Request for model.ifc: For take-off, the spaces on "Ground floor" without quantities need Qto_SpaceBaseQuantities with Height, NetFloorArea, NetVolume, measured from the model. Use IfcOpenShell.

First a look at what the model holds.

```python
import ifcopenshell
import ifcopenshell.util.element
import ifcopenshell.util.unit

model = ifcopenshell.open("model.ifc")
print(model.schema)
for unit_type in ("LENGTHUNIT", "AREAUNIT", "VOLUMEUNIT"):
    print(unit_type, ifcopenshell.util.unit.calculate_unit_scale(model, unit_type))
storey = next(s for s in model.by_type("IfcBuildingStorey") if s.Name == "Ground floor")
spaces = [e for e in ifcopenshell.util.element.get_decomposition(storey) if e.is_a("IfcSpace")]
for e in sorted(spaces, key=lambda e: e.id()):
    print(e.id(), e.is_a(), e.Name, list(ifcopenshell.util.element.get_psets(e, qtos_only=True)), sep=" | ")
```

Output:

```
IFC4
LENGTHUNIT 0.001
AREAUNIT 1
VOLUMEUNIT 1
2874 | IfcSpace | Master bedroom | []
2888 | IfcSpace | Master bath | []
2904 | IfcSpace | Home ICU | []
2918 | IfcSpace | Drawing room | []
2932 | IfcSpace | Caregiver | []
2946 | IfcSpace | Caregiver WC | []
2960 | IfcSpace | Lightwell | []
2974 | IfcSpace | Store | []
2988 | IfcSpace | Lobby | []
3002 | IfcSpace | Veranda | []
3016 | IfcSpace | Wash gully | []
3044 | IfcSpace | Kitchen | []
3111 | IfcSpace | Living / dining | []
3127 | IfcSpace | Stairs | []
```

```python
import ifcopenshell
import ifcopenshell.api.pset
import ifcopenshell.geom
import ifcopenshell.util.element
import ifcopenshell.util.shape
import ifcopenshell.util.unit

model = ifcopenshell.open("model.ifc")
unit_scale = ifcopenshell.util.unit.calculate_unit_scale(model)
area_scale = ifcopenshell.util.unit.calculate_unit_scale(model, "AREAUNIT")
volume_scale = ifcopenshell.util.unit.calculate_unit_scale(model, "VOLUMEUNIT")
settings = ifcopenshell.geom.settings()

storey = next(s for s in model.by_type("IfcBuildingStorey") if s.Name == "Ground floor")
spaces = [e for e in ifcopenshell.util.element.get_decomposition(storey) if e.is_a("IfcSpace")]

for e in sorted(spaces, key=lambda e: e.id()):
    if ifcopenshell.util.element.get_psets(e, qtos_only=True, should_inherit=False):
        continue
    # Geometry comes back in metres, in the element's own axes.
    shape = ifcopenshell.geom.create_shape(settings, e)
    values = {
        "Height": ifcopenshell.util.shape.get_z(shape.geometry) / unit_scale,
        "NetFloorArea": ifcopenshell.util.shape.get_footprint_area(shape.geometry) / area_scale,
        "NetVolume": ifcopenshell.util.shape.get_volume(shape.geometry) / volume_scale,
    }
    qto = ifcopenshell.api.pset.add_qto(model, product=e, name="Qto_SpaceBaseQuantities")
    ifcopenshell.api.pset.edit_qto(model, qto=qto, properties=values)
    print(e.id(), {k: round(v, 3) for k, v in values.items()})

model.write("model_updated.ifc")
```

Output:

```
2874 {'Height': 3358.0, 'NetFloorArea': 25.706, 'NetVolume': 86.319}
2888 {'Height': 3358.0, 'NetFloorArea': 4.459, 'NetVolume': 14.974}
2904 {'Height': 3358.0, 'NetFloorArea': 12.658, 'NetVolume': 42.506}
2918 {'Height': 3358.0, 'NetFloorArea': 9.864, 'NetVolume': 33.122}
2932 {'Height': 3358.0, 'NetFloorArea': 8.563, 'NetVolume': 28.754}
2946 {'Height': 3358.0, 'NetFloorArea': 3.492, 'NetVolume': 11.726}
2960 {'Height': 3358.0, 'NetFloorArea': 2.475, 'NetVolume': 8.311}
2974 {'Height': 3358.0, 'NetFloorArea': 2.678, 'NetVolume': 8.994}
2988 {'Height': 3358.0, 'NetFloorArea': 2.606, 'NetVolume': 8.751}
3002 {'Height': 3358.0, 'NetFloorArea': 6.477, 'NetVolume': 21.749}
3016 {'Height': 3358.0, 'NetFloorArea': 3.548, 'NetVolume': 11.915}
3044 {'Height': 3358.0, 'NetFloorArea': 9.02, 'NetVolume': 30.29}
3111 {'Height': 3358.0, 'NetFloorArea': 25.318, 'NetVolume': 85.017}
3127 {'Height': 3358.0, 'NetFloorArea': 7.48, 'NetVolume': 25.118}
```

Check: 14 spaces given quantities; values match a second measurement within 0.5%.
